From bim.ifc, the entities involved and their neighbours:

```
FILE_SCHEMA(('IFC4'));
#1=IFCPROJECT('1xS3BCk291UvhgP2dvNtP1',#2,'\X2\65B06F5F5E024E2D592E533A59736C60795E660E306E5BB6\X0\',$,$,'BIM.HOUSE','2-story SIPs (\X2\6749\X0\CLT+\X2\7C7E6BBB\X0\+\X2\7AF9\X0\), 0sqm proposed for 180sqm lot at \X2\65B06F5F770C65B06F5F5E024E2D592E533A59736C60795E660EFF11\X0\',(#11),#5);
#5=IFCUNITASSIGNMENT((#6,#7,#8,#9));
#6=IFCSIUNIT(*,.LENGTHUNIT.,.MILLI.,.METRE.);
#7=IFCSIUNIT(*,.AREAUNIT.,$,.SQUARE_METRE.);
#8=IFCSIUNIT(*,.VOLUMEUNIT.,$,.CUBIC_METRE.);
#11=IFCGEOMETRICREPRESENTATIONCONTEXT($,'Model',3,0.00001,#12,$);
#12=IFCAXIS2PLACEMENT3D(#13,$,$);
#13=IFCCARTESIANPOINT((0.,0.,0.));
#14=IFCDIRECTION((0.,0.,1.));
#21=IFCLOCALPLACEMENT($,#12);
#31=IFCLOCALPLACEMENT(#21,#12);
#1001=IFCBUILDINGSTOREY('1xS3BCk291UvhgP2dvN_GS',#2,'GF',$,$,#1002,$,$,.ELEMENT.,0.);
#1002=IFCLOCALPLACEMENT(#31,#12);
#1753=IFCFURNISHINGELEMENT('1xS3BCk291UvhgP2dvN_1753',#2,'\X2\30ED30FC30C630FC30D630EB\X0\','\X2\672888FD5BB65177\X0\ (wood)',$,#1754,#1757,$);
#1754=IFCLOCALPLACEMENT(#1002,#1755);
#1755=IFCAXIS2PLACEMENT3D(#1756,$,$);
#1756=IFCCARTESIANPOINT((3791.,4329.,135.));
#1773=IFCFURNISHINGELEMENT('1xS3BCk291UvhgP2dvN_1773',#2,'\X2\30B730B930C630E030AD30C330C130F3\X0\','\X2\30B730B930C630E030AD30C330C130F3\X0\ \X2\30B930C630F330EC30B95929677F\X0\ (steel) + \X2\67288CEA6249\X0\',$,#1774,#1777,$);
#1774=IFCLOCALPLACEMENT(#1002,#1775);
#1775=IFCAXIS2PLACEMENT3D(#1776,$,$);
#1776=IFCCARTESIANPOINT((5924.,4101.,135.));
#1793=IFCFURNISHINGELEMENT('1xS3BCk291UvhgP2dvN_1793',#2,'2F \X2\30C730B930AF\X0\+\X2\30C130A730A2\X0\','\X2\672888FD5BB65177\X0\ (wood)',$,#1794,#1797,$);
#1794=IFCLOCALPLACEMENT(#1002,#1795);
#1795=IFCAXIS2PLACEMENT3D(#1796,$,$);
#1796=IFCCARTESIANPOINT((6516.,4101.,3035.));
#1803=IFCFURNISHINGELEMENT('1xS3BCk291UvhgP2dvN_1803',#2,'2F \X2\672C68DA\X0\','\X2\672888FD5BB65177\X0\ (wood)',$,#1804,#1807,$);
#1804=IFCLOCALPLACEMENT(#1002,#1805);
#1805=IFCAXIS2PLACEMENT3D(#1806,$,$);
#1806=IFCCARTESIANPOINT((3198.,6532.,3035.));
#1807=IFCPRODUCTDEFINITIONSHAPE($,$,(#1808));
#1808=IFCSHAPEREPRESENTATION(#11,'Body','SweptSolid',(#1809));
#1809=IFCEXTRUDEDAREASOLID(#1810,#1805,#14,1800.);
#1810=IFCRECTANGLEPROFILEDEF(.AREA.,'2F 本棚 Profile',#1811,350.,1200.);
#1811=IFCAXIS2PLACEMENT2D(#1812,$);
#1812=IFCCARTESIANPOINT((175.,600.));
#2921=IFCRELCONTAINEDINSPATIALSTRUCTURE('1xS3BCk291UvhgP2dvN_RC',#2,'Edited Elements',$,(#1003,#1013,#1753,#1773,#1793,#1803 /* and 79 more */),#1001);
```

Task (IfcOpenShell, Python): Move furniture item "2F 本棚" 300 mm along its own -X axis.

```python
import ifcopenshell
import ifcopenshell.api.geometry
import ifcopenshell.util.placement
import ifcopenshell.util.unit

model = ifcopenshell.open("bim.ifc")
unit_scale = ifcopenshell.util.unit.calculate_unit_scale(model)

item = model.by_id(1803)
matrix = ifcopenshell.util.placement.get_local_placement(item.ObjectPlacement)
matrix[:3, 3] -= matrix[:3, 0] * 0.3 / unit_scale
ifcopenshell.api.geometry.edit_object_placement(model, product=item, matrix=matrix, is_si=False)

print(ifcopenshell.util.placement.get_local_placement(item.ObjectPlacement).round(3) + 0.0)

model.write("bim_edited.ifc")
```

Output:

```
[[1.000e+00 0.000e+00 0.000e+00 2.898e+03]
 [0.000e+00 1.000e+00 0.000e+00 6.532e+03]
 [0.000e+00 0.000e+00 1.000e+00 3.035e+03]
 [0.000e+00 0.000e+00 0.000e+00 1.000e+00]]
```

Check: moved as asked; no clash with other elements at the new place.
